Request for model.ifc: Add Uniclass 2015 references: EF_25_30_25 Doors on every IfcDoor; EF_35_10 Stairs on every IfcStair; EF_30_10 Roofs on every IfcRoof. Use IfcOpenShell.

First a look at what the model holds.

```python
import ifcopenshell

model = ifcopenshell.open("model.ifc")
print(model.schema)
print("classifications:", [c.Name for c in model.by_type("IfcClassification")])
for ifc_class in ("IfcDoor", "IfcRoof", "IfcStair", "IfcWall", "IfcWindow"):
    print(ifc_class, len(model.by_type(ifc_class)))
```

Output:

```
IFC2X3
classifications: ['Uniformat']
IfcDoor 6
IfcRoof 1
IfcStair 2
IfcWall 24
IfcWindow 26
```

```python
import ifcopenshell
import ifcopenshell.api.classification

model = ifcopenshell.open("model.ifc")

# IFC2X3 requires Source and Edition and has no link from the project to the system.
system = model.create_entity("IfcClassification", Source="NBS", Edition="2015", Name="Uniclass 2015")

codes = {
    "IfcDoor": ("EF_25_30_25", "Doors"),
    "IfcStair": ("EF_35_10", "Stairs"),
    "IfcRoof": ("EF_30_10", "Roofs"),
}
for ifc_class, (code, name) in codes.items():
    products = model.by_type(ifc_class)
    ifcopenshell.api.classification.add_reference(
        model, products=products, classification=system, identification=code, name=name
    )
    print(code, len(products))

model.write("model-out.ifc")
```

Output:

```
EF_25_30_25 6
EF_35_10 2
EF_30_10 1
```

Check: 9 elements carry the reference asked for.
